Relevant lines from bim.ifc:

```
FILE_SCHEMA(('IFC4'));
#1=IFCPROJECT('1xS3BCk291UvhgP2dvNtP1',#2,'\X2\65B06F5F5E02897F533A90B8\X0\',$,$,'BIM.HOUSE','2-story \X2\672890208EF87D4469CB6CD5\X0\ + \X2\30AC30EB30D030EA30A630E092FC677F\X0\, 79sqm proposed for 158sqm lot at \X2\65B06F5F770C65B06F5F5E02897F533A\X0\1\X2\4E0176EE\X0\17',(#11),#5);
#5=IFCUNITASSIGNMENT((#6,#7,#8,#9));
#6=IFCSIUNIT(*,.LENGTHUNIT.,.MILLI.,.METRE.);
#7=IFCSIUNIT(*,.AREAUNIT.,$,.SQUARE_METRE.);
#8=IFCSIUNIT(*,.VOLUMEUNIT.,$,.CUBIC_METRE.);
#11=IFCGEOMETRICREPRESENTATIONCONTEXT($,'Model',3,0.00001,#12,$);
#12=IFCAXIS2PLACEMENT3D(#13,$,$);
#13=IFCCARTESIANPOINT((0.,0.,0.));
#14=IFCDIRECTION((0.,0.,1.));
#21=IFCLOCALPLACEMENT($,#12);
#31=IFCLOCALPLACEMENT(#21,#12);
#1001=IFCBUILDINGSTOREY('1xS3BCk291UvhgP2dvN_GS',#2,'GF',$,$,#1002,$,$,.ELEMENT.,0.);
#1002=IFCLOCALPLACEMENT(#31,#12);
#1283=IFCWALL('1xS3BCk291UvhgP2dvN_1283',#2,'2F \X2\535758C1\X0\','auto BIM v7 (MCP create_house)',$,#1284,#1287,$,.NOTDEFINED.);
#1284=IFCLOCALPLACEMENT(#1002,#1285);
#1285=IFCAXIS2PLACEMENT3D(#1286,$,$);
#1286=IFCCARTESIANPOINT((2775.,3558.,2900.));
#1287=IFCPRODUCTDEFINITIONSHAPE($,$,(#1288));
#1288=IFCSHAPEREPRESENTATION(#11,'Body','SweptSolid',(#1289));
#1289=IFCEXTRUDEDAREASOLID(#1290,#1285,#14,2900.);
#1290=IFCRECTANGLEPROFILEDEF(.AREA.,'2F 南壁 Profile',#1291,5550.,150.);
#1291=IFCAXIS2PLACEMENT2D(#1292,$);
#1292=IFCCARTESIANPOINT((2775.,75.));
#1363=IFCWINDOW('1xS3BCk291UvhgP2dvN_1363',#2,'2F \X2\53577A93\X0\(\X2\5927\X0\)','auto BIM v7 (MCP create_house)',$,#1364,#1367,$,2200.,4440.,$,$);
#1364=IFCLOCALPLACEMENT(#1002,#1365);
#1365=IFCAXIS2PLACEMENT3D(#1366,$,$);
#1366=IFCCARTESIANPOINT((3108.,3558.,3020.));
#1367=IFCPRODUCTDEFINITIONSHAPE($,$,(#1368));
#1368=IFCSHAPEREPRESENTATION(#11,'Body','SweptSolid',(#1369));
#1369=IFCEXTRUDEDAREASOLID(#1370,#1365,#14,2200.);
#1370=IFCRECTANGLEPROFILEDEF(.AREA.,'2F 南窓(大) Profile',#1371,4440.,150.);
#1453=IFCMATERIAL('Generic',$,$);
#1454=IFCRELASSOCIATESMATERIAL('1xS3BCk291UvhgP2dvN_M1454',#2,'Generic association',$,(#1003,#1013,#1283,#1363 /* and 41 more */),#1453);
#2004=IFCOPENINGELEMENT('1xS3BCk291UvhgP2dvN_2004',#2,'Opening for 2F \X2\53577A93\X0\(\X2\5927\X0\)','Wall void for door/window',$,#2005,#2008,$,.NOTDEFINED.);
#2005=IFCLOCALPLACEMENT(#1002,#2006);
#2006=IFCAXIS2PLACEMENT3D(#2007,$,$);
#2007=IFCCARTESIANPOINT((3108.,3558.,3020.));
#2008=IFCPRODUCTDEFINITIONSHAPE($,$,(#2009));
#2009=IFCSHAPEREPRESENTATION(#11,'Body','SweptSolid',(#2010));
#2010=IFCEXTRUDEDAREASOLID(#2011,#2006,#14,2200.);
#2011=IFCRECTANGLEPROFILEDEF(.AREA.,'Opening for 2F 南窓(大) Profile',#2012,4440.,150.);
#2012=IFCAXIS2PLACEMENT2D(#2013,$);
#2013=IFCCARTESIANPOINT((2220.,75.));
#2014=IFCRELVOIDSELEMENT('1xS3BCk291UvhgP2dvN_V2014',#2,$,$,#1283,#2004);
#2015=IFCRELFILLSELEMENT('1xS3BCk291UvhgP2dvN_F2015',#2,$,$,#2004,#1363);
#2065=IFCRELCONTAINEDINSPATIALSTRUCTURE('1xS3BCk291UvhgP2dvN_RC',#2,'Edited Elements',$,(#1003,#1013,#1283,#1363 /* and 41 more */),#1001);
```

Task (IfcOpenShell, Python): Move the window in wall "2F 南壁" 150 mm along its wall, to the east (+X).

```python
import ifcopenshell
import ifcopenshell.api.geometry
import ifcopenshell.util.placement
import ifcopenshell.util.unit

model = ifcopenshell.open("bim.ifc")
unit_scale = ifcopenshell.util.unit.calculate_unit_scale(model)

window = model.by_guid("1xS3BCk291UvhgP2dvN_1363")
opening = window.FillsVoids[0].RelatingOpeningElement
wall = opening.VoidsElements[0].RelatingBuildingElement

wall_matrix = ifcopenshell.util.placement.get_local_placement(wall.ObjectPlacement)
shift = wall_matrix[:3, 0] * 0.15 / unit_scale
before = ifcopenshell.util.placement.get_local_placement(window.ObjectPlacement)[:3, 3].copy()

# The window is not placed relative to its opening, so move both.
for product in (opening, window):
    matrix = ifcopenshell.util.placement.get_local_placement(product.ObjectPlacement)
    matrix[:3, 3] += shift
    ifcopenshell.api.geometry.edit_object_placement(model, product=product, matrix=matrix, is_si=False)

after = ifcopenshell.util.placement.get_local_placement(window.ObjectPlacement)[:3, 3]
print("window moved by", (after - before).round(3) + 0.0)

model.write("bim_updated.ifc")
```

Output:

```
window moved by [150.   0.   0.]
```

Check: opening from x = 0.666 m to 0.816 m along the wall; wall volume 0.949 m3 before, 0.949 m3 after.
